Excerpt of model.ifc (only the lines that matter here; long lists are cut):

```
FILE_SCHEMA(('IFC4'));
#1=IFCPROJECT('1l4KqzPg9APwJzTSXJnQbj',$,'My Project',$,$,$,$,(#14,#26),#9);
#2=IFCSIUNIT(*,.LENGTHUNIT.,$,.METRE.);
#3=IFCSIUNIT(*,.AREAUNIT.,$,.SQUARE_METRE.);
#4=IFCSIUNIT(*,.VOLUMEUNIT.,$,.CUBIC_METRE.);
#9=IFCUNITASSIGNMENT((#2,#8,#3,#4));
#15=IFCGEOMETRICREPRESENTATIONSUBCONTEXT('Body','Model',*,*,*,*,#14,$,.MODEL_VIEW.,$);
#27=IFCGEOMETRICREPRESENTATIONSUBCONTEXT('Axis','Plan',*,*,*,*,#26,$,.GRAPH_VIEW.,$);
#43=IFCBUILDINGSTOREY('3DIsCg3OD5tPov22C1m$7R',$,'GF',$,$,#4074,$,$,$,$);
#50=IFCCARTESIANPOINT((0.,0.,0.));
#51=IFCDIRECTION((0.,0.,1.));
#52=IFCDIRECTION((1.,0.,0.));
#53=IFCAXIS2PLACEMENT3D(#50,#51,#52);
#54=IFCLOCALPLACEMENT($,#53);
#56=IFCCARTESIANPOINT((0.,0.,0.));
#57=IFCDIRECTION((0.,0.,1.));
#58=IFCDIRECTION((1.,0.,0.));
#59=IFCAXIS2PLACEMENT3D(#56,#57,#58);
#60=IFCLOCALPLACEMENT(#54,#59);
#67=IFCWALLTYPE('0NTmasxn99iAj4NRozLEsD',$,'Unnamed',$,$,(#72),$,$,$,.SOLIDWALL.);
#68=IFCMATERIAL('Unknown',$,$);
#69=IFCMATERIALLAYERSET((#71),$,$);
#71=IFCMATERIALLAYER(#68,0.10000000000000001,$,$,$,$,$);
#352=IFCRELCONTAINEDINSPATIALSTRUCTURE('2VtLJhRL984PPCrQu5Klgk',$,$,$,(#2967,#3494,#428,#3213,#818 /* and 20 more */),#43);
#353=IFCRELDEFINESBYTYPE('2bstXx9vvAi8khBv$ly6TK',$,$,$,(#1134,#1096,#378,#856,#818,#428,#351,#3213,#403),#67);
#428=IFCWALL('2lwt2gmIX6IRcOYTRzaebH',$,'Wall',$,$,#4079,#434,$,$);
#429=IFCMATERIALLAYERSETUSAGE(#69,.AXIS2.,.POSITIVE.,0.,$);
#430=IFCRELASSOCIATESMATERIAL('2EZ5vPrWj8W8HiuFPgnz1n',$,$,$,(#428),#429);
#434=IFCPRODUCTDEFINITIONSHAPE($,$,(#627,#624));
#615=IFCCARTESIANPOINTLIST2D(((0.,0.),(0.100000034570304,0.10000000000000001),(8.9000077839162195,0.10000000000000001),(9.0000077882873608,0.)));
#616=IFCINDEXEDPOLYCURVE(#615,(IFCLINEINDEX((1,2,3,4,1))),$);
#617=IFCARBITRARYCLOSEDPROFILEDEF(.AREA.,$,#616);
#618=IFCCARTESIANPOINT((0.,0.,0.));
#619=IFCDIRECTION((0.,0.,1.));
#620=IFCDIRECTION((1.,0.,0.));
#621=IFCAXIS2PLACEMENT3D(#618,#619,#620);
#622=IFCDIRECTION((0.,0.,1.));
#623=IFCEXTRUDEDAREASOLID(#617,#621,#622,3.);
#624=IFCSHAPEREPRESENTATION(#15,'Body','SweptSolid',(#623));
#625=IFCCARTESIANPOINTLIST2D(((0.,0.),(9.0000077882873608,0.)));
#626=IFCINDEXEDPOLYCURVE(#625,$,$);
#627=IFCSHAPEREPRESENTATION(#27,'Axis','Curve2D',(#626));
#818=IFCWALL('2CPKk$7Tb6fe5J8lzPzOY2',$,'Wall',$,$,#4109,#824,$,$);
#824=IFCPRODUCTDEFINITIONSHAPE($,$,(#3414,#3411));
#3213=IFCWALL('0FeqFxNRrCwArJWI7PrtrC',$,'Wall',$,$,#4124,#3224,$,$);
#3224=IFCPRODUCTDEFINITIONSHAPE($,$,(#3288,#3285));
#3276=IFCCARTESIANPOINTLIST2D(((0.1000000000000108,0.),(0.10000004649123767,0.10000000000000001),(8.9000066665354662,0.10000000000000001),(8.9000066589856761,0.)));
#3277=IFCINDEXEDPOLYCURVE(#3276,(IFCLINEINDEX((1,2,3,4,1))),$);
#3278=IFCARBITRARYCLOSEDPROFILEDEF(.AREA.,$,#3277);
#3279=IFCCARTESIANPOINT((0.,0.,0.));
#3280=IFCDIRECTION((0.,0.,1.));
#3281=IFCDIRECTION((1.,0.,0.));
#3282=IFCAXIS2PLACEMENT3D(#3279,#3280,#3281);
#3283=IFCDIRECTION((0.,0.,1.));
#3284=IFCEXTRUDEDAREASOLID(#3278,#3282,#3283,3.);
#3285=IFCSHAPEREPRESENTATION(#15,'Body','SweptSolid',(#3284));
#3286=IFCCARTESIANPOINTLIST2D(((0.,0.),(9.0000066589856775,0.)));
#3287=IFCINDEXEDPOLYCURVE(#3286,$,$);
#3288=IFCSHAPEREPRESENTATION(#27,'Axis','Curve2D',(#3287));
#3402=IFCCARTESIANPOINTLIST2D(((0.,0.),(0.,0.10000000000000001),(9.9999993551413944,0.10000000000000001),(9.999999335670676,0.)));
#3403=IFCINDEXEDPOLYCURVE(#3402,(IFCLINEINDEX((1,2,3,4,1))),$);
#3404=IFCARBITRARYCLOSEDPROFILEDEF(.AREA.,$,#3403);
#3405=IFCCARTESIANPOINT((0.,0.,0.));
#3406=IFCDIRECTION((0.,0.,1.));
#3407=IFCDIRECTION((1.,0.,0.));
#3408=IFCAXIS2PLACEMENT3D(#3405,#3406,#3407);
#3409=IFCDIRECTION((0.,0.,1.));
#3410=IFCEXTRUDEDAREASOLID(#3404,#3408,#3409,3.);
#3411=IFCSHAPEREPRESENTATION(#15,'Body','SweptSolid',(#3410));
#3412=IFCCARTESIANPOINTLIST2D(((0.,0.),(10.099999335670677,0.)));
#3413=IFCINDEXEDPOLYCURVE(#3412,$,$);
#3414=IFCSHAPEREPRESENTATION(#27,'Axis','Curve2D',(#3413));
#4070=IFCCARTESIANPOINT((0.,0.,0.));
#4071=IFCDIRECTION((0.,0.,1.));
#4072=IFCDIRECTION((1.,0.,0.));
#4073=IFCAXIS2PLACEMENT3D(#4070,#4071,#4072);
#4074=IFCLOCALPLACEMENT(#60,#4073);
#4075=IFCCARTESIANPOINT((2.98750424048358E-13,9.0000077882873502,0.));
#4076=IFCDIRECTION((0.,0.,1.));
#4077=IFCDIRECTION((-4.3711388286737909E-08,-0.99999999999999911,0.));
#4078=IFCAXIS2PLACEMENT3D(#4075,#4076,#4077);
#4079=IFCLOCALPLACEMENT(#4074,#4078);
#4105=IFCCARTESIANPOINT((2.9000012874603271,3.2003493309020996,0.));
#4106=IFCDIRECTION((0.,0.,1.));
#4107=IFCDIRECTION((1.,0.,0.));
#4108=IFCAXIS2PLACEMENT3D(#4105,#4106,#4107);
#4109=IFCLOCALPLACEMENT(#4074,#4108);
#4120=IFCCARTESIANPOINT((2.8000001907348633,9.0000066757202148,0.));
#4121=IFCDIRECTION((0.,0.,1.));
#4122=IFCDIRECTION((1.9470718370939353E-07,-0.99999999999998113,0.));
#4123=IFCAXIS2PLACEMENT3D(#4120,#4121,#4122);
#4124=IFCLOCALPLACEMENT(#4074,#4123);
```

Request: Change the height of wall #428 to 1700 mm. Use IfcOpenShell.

```python
import ifcopenshell
import ifcopenshell.geom
import ifcopenshell.util.representation
import ifcopenshell.util.shape
import ifcopenshell.util.unit

model = ifcopenshell.open("model.ifc")
unit_scale = ifcopenshell.util.unit.calculate_unit_scale(model)
settings = ifcopenshell.geom.settings()


def volume(element):
    """Net volume in cubic metres, openings subtracted."""
    shape = ifcopenshell.geom.create_shape(settings, element)
    return ifcopenshell.util.shape.get_volume(shape.geometry)


wall = model.by_guid("2lwt2gmIX6IRcOYTRzaebH")
before = volume(wall)

body = ifcopenshell.util.representation.get_representation(wall, "Model", "Body")
solid = body.Items[0]
old_height = solid.Depth
solid.Depth = 1.7 / unit_scale
after = volume(wall)

print(f"height {old_height:g} -> {solid.Depth:g}, volume {before:.3f} -> {after:.3f} m3")

model.write("model_rev.ifc")
```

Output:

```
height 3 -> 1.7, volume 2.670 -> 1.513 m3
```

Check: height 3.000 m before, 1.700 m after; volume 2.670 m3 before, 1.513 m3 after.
